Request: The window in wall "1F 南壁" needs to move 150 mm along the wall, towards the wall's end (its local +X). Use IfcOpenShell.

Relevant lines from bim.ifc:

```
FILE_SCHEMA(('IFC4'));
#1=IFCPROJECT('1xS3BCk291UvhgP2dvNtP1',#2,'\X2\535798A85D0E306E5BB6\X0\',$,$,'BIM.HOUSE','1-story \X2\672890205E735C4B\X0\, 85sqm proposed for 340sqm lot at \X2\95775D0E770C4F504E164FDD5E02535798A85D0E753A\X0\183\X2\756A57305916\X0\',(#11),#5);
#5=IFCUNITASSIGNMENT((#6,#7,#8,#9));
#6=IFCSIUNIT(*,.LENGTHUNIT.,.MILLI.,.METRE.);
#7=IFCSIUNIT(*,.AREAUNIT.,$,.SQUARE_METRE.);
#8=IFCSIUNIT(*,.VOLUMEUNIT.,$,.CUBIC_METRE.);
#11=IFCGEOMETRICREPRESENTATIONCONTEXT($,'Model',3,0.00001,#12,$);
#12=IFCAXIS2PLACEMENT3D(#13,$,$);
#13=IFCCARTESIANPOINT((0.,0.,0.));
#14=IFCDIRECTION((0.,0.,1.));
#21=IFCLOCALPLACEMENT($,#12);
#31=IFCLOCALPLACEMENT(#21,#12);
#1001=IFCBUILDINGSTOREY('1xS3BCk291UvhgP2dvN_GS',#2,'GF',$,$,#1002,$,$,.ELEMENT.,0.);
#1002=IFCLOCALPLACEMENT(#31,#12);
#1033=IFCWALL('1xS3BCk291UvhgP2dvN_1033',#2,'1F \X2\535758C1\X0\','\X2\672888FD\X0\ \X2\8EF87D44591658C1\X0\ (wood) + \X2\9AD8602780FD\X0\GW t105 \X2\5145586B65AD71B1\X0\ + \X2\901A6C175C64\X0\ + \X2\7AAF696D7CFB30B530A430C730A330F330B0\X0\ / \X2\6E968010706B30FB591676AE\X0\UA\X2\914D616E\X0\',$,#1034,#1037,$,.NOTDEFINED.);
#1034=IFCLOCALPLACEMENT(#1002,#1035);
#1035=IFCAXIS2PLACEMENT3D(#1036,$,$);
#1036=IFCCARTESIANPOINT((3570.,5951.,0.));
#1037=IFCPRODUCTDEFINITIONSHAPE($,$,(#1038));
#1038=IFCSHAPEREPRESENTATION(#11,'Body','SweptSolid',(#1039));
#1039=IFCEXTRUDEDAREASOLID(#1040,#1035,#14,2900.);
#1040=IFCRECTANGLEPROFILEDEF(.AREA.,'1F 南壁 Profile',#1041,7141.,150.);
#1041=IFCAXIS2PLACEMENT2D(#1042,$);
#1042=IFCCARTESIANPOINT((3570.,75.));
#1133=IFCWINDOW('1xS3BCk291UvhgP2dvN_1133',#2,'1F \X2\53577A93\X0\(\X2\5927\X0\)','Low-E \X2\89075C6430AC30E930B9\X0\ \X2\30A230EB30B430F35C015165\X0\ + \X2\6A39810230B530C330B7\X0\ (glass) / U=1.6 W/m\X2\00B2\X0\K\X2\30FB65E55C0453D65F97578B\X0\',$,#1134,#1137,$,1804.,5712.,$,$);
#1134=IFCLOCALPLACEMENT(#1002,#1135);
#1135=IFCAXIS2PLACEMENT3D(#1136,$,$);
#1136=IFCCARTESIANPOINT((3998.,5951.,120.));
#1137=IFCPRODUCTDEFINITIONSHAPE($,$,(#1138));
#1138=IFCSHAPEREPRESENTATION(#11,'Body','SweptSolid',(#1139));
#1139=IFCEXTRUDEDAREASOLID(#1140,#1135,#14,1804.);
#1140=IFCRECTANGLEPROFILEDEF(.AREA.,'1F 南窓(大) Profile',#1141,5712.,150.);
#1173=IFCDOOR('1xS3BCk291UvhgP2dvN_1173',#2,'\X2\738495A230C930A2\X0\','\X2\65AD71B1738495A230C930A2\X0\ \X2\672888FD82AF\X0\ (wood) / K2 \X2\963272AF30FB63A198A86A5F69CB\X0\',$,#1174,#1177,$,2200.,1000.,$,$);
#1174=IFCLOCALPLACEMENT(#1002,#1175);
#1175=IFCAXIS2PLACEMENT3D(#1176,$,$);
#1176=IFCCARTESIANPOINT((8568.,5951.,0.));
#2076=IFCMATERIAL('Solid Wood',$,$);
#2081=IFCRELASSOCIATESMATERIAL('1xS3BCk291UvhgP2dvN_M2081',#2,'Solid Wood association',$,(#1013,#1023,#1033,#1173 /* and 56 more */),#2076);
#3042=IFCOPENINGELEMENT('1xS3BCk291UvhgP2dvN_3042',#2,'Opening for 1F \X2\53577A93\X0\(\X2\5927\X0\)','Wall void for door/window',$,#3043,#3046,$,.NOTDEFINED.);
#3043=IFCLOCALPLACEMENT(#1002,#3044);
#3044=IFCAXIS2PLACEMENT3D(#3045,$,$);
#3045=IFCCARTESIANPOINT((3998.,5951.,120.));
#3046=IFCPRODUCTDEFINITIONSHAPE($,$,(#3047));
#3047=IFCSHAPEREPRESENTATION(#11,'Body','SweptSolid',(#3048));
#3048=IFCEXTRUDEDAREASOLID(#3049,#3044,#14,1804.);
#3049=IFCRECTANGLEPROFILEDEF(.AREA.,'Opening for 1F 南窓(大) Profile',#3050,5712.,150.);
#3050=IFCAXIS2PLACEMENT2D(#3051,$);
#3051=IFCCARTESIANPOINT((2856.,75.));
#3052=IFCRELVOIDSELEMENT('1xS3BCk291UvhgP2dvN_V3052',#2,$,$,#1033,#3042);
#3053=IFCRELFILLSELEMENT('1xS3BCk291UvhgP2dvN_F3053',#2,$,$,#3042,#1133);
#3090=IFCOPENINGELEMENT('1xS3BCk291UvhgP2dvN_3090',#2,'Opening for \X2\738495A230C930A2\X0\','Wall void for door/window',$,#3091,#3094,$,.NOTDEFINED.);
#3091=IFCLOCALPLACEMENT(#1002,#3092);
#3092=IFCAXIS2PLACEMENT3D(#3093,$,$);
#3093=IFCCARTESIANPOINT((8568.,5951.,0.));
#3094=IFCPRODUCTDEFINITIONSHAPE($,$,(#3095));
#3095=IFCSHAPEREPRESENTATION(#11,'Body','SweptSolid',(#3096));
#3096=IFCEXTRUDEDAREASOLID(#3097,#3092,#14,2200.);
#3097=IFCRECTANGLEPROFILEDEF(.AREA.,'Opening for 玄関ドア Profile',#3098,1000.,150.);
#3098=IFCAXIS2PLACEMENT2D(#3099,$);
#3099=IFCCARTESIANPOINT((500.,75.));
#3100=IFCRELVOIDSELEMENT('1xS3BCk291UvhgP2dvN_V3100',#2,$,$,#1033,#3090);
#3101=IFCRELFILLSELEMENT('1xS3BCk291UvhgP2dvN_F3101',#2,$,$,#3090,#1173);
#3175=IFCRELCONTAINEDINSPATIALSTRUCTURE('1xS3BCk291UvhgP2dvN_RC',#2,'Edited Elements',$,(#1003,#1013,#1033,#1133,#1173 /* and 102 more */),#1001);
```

```python
import ifcopenshell
import ifcopenshell.api.geometry
import ifcopenshell.util.placement
import ifcopenshell.util.unit

model = ifcopenshell.open("bim.ifc")
unit_scale = ifcopenshell.util.unit.calculate_unit_scale(model)

window = model.by_guid("1xS3BCk291UvhgP2dvN_1133")
opening = window.FillsVoids[0].RelatingOpeningElement
wall = opening.VoidsElements[0].RelatingBuildingElement

wall_matrix = ifcopenshell.util.placement.get_local_placement(wall.ObjectPlacement)
shift = wall_matrix[:3, 0] * 0.15 / unit_scale
before = ifcopenshell.util.placement.get_local_placement(window.ObjectPlacement)[:3, 3].copy()

# The window is not placed relative to its opening, so move both.
for product in (opening, window):
    matrix = ifcopenshell.util.placement.get_local_placement(product.ObjectPlacement)
    matrix[:3, 3] += shift
    ifcopenshell.api.geometry.edit_object_placement(model, product=product, matrix=matrix, is_si=False)

after = ifcopenshell.util.placement.get_local_placement(window.ObjectPlacement)[:3, 3]
print("window moved by", (after - before).round(3) + 0.0)

model.write("bim_v2.ifc")
```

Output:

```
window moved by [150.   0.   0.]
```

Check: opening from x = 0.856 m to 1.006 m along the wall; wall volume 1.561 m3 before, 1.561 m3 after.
